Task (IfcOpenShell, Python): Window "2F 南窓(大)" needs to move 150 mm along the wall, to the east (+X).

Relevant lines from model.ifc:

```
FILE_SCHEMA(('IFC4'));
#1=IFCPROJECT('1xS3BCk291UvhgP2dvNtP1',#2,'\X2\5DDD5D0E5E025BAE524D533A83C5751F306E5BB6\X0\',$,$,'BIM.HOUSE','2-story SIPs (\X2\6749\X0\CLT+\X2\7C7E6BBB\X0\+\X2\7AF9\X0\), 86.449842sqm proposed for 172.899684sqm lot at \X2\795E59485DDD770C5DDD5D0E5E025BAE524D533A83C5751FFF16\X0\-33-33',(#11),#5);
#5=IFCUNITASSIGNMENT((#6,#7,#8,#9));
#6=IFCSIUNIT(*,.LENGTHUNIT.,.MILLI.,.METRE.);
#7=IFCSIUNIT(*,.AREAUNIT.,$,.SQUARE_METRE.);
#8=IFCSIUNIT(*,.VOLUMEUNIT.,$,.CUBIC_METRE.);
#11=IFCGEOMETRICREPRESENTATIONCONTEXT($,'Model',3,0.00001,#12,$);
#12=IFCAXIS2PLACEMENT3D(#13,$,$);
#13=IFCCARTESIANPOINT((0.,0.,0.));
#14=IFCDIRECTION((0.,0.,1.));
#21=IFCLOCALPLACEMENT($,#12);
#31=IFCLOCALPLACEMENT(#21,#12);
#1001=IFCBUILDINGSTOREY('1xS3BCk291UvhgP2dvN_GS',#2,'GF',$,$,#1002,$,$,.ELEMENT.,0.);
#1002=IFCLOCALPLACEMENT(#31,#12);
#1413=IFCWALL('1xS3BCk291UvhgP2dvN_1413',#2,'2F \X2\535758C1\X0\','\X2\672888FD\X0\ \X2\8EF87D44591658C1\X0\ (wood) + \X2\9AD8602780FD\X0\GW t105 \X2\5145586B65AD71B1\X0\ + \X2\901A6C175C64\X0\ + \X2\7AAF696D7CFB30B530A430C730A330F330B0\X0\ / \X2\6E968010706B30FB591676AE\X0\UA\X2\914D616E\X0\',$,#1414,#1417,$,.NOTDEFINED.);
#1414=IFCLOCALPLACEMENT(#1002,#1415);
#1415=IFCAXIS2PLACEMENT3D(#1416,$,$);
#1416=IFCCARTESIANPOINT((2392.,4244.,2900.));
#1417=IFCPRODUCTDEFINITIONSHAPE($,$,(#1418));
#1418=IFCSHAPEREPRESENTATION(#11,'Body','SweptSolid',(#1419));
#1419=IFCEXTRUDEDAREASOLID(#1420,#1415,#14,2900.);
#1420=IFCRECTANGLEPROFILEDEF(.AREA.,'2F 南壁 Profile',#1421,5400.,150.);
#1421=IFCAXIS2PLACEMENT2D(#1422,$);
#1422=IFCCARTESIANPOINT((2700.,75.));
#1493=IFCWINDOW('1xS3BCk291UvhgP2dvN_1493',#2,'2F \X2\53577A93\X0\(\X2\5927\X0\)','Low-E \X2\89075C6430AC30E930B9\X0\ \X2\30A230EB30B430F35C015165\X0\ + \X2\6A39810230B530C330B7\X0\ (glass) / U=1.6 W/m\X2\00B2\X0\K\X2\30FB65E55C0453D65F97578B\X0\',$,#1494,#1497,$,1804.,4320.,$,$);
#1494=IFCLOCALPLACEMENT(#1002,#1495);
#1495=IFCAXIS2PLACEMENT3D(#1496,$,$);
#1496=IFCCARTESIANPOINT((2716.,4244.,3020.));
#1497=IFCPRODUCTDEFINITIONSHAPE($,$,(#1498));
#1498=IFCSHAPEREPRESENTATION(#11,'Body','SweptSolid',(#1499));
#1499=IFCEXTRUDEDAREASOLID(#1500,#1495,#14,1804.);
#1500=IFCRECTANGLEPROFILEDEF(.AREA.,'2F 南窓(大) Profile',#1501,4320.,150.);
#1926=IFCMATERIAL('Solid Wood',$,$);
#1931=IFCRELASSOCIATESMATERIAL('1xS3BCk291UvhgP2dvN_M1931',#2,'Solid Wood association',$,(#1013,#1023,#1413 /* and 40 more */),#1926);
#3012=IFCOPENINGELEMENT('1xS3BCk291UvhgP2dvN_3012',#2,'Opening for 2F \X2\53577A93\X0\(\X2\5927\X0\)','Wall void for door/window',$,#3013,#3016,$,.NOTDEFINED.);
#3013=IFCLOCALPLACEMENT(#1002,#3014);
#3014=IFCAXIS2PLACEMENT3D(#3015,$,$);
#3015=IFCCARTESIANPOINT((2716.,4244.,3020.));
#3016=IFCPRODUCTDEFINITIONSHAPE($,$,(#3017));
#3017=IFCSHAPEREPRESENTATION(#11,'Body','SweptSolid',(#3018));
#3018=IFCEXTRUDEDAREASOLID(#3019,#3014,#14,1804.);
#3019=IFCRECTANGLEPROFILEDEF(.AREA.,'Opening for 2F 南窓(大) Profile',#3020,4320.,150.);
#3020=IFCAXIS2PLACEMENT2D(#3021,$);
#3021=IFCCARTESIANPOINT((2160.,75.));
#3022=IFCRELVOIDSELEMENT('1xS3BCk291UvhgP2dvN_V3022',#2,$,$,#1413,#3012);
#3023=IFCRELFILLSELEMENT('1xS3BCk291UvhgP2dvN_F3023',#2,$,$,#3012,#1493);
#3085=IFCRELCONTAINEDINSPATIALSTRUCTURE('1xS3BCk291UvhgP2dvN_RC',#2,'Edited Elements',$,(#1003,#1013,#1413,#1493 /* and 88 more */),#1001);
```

```python
import ifcopenshell
import ifcopenshell.api.geometry
import ifcopenshell.util.placement
import ifcopenshell.util.unit

model = ifcopenshell.open("model.ifc")
unit_scale = ifcopenshell.util.unit.calculate_unit_scale(model)

window = model.by_id(1493)
opening = window.FillsVoids[0].RelatingOpeningElement
wall = opening.VoidsElements[0].RelatingBuildingElement

wall_matrix = ifcopenshell.util.placement.get_local_placement(wall.ObjectPlacement)
shift = wall_matrix[:3, 0] * 0.15 / unit_scale
before = ifcopenshell.util.placement.get_local_placement(window.ObjectPlacement)[:3, 3].copy()

# The window is not placed relative to its opening, so move both.
for product in (opening, window):
    matrix = ifcopenshell.util.placement.get_local_placement(product.ObjectPlacement)
    matrix[:3, 3] += shift
    ifcopenshell.api.geometry.edit_object_placement(model, product=product, matrix=matrix, is_si=False)

after = ifcopenshell.util.placement.get_local_placement(window.ObjectPlacement)[:3, 3]
print("window moved by", (after - before).round(3) + 0.0)

model.write("model_v2.ifc")
```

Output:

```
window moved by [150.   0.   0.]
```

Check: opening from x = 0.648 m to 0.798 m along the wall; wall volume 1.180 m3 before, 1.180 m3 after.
